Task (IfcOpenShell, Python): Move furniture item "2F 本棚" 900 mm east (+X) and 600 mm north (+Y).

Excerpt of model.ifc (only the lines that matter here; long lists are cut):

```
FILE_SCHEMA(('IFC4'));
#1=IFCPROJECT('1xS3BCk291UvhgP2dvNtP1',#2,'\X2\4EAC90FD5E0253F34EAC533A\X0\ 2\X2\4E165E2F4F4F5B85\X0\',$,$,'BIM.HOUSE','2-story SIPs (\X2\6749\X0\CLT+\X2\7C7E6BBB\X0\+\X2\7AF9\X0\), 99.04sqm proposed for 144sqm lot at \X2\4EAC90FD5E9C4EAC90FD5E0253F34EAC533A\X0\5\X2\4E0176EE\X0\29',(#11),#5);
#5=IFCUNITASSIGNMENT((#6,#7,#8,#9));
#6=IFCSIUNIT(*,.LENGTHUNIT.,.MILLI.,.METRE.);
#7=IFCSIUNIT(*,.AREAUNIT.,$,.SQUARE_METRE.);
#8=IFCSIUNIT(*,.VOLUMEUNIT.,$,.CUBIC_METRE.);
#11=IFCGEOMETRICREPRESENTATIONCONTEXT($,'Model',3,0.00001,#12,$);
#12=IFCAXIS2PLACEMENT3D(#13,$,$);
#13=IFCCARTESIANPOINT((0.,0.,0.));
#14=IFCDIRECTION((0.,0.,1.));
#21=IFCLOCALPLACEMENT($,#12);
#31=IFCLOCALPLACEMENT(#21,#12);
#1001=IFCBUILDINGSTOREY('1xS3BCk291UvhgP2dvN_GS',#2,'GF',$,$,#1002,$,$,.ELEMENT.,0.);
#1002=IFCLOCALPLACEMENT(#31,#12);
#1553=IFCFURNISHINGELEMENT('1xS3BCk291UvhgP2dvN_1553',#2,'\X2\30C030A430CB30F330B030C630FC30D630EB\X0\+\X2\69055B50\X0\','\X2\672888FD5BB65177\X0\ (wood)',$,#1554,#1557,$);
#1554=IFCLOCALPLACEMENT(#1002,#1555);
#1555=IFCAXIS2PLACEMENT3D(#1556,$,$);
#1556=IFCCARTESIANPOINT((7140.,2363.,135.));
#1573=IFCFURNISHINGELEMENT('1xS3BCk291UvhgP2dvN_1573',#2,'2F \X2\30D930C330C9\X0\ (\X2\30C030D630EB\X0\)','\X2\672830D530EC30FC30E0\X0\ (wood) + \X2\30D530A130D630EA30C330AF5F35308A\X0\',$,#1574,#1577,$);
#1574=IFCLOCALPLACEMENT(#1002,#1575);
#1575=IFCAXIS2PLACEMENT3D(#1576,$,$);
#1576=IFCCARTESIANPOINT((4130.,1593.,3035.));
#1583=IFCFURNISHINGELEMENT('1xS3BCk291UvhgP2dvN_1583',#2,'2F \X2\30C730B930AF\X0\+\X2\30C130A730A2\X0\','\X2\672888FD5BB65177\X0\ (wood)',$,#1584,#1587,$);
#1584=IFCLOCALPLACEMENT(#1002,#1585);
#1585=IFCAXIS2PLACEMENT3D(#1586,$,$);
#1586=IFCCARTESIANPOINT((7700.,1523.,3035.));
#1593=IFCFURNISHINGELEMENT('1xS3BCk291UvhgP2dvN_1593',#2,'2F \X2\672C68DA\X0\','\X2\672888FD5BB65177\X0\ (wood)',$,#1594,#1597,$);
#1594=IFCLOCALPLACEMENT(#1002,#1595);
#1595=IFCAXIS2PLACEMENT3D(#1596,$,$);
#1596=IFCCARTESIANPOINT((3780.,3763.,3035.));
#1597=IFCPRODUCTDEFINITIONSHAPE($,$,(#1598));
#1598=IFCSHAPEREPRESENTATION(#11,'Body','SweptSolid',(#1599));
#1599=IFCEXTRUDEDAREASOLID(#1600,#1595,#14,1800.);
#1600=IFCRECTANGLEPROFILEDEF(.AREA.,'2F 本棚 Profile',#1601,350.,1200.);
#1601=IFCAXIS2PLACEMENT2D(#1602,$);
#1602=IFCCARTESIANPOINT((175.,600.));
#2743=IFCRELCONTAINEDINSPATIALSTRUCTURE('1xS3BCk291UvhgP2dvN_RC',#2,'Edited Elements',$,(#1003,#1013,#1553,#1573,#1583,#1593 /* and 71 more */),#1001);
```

```python
import ifcopenshell
import ifcopenshell.api.geometry
import ifcopenshell.util.placement
import ifcopenshell.util.unit

model = ifcopenshell.open("model.ifc")
unit_scale = ifcopenshell.util.unit.calculate_unit_scale(model)

item = model.by_id(1593)
matrix = ifcopenshell.util.placement.get_local_placement(item.ObjectPlacement)
matrix[0, 3] += 0.9 / unit_scale
matrix[1, 3] += 0.6 / unit_scale
ifcopenshell.api.geometry.edit_object_placement(model, product=item, matrix=matrix, is_si=False)

print(ifcopenshell.util.placement.get_local_placement(item.ObjectPlacement).round(3) + 0.0)

model.write("model-out.ifc")
```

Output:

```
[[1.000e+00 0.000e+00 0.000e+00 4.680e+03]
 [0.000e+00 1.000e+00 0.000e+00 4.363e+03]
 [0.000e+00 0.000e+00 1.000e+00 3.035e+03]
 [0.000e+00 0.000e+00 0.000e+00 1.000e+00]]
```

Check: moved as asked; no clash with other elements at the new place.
